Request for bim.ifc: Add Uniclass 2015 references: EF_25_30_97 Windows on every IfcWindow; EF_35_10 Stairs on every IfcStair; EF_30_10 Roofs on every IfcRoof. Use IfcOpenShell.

First a look at what the model holds.

```python
import ifcopenshell

model = ifcopenshell.open("bim.ifc")
print(model.schema)
print("classifications:", [c.Name for c in model.by_type("IfcClassification")])
for ifc_class in ("IfcDoor", "IfcRoof", "IfcStair", "IfcWall", "IfcWindow"):
    print(ifc_class, len(model.by_type(ifc_class)))
```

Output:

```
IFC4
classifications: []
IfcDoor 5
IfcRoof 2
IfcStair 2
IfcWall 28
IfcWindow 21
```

```python
import ifcopenshell
import ifcopenshell.api.classification

model = ifcopenshell.open("bim.ifc")

system = ifcopenshell.api.classification.add_classification(model, classification="Uniclass 2015")

codes = {
    "IfcWindow": ("EF_25_30_97", "Windows"),
    "IfcStair": ("EF_35_10", "Stairs"),
    "IfcRoof": ("EF_30_10", "Roofs"),
}
for ifc_class, (code, name) in codes.items():
    products = model.by_type(ifc_class)
    ifcopenshell.api.classification.add_reference(
        model, products=products, classification=system, identification=code, name=name
    )
    print(code, len(products))

model.write("bim_updated.ifc")
```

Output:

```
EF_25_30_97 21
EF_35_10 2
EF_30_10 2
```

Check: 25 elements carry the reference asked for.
